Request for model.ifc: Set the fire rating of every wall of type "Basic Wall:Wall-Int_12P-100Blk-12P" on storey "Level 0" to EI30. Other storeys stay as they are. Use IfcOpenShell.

First a look at what the model holds.

```python
import ifcopenshell
import ifcopenshell.util.element

model = ifcopenshell.open("model.ifc")
print(model.schema)
storey = next(s for s in model.by_type("IfcBuildingStorey") if s.Name == "Level 0")
walls = [e for e in ifcopenshell.util.element.get_decomposition(storey) if e.is_a("IfcWall")]
seen = {}
for e in walls:
    element_type = ifcopenshell.util.element.get_type(e)
    key = (element_type.Name if element_type != e and element_type else None, ifcopenshell.util.element.get_pset(e, "Pset_WallCommon", "FireRating"))
    seen[key] = seen.get(key, 0) + 1
for (name, value), count in sorted(seen.items(), key=str):
    print(count, "x", name, "|", value)
```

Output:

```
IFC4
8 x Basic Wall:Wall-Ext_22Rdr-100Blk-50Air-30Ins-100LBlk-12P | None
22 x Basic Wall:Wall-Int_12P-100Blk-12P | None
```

```python
import ifcopenshell
import ifcopenshell.api.pset
import ifcopenshell.util.element

model = ifcopenshell.open("model.ifc")

storey = next(s for s in model.by_type("IfcBuildingStorey") if s.Name == "Level 0")
walls = [e for e in ifcopenshell.util.element.get_decomposition(storey) if e.is_a("IfcWall")]

count = 0
for e in walls:
    element_type = ifcopenshell.util.element.get_type(e)
    if element_type in (None, e) or element_type.Name != "Basic Wall:Wall-Int_12P-100Blk-12P":
        continue
    # add_pset returns the element's existing set when there is one.
    pset = ifcopenshell.api.pset.add_pset(model, product=e, name="Pset_WallCommon")
    ifcopenshell.api.pset.edit_pset(model, pset=pset, properties={"FireRating": "EI30"})
    count += 1

print(count, "walls updated")

model.write("model_rev.ifc")
```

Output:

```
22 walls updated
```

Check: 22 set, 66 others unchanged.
